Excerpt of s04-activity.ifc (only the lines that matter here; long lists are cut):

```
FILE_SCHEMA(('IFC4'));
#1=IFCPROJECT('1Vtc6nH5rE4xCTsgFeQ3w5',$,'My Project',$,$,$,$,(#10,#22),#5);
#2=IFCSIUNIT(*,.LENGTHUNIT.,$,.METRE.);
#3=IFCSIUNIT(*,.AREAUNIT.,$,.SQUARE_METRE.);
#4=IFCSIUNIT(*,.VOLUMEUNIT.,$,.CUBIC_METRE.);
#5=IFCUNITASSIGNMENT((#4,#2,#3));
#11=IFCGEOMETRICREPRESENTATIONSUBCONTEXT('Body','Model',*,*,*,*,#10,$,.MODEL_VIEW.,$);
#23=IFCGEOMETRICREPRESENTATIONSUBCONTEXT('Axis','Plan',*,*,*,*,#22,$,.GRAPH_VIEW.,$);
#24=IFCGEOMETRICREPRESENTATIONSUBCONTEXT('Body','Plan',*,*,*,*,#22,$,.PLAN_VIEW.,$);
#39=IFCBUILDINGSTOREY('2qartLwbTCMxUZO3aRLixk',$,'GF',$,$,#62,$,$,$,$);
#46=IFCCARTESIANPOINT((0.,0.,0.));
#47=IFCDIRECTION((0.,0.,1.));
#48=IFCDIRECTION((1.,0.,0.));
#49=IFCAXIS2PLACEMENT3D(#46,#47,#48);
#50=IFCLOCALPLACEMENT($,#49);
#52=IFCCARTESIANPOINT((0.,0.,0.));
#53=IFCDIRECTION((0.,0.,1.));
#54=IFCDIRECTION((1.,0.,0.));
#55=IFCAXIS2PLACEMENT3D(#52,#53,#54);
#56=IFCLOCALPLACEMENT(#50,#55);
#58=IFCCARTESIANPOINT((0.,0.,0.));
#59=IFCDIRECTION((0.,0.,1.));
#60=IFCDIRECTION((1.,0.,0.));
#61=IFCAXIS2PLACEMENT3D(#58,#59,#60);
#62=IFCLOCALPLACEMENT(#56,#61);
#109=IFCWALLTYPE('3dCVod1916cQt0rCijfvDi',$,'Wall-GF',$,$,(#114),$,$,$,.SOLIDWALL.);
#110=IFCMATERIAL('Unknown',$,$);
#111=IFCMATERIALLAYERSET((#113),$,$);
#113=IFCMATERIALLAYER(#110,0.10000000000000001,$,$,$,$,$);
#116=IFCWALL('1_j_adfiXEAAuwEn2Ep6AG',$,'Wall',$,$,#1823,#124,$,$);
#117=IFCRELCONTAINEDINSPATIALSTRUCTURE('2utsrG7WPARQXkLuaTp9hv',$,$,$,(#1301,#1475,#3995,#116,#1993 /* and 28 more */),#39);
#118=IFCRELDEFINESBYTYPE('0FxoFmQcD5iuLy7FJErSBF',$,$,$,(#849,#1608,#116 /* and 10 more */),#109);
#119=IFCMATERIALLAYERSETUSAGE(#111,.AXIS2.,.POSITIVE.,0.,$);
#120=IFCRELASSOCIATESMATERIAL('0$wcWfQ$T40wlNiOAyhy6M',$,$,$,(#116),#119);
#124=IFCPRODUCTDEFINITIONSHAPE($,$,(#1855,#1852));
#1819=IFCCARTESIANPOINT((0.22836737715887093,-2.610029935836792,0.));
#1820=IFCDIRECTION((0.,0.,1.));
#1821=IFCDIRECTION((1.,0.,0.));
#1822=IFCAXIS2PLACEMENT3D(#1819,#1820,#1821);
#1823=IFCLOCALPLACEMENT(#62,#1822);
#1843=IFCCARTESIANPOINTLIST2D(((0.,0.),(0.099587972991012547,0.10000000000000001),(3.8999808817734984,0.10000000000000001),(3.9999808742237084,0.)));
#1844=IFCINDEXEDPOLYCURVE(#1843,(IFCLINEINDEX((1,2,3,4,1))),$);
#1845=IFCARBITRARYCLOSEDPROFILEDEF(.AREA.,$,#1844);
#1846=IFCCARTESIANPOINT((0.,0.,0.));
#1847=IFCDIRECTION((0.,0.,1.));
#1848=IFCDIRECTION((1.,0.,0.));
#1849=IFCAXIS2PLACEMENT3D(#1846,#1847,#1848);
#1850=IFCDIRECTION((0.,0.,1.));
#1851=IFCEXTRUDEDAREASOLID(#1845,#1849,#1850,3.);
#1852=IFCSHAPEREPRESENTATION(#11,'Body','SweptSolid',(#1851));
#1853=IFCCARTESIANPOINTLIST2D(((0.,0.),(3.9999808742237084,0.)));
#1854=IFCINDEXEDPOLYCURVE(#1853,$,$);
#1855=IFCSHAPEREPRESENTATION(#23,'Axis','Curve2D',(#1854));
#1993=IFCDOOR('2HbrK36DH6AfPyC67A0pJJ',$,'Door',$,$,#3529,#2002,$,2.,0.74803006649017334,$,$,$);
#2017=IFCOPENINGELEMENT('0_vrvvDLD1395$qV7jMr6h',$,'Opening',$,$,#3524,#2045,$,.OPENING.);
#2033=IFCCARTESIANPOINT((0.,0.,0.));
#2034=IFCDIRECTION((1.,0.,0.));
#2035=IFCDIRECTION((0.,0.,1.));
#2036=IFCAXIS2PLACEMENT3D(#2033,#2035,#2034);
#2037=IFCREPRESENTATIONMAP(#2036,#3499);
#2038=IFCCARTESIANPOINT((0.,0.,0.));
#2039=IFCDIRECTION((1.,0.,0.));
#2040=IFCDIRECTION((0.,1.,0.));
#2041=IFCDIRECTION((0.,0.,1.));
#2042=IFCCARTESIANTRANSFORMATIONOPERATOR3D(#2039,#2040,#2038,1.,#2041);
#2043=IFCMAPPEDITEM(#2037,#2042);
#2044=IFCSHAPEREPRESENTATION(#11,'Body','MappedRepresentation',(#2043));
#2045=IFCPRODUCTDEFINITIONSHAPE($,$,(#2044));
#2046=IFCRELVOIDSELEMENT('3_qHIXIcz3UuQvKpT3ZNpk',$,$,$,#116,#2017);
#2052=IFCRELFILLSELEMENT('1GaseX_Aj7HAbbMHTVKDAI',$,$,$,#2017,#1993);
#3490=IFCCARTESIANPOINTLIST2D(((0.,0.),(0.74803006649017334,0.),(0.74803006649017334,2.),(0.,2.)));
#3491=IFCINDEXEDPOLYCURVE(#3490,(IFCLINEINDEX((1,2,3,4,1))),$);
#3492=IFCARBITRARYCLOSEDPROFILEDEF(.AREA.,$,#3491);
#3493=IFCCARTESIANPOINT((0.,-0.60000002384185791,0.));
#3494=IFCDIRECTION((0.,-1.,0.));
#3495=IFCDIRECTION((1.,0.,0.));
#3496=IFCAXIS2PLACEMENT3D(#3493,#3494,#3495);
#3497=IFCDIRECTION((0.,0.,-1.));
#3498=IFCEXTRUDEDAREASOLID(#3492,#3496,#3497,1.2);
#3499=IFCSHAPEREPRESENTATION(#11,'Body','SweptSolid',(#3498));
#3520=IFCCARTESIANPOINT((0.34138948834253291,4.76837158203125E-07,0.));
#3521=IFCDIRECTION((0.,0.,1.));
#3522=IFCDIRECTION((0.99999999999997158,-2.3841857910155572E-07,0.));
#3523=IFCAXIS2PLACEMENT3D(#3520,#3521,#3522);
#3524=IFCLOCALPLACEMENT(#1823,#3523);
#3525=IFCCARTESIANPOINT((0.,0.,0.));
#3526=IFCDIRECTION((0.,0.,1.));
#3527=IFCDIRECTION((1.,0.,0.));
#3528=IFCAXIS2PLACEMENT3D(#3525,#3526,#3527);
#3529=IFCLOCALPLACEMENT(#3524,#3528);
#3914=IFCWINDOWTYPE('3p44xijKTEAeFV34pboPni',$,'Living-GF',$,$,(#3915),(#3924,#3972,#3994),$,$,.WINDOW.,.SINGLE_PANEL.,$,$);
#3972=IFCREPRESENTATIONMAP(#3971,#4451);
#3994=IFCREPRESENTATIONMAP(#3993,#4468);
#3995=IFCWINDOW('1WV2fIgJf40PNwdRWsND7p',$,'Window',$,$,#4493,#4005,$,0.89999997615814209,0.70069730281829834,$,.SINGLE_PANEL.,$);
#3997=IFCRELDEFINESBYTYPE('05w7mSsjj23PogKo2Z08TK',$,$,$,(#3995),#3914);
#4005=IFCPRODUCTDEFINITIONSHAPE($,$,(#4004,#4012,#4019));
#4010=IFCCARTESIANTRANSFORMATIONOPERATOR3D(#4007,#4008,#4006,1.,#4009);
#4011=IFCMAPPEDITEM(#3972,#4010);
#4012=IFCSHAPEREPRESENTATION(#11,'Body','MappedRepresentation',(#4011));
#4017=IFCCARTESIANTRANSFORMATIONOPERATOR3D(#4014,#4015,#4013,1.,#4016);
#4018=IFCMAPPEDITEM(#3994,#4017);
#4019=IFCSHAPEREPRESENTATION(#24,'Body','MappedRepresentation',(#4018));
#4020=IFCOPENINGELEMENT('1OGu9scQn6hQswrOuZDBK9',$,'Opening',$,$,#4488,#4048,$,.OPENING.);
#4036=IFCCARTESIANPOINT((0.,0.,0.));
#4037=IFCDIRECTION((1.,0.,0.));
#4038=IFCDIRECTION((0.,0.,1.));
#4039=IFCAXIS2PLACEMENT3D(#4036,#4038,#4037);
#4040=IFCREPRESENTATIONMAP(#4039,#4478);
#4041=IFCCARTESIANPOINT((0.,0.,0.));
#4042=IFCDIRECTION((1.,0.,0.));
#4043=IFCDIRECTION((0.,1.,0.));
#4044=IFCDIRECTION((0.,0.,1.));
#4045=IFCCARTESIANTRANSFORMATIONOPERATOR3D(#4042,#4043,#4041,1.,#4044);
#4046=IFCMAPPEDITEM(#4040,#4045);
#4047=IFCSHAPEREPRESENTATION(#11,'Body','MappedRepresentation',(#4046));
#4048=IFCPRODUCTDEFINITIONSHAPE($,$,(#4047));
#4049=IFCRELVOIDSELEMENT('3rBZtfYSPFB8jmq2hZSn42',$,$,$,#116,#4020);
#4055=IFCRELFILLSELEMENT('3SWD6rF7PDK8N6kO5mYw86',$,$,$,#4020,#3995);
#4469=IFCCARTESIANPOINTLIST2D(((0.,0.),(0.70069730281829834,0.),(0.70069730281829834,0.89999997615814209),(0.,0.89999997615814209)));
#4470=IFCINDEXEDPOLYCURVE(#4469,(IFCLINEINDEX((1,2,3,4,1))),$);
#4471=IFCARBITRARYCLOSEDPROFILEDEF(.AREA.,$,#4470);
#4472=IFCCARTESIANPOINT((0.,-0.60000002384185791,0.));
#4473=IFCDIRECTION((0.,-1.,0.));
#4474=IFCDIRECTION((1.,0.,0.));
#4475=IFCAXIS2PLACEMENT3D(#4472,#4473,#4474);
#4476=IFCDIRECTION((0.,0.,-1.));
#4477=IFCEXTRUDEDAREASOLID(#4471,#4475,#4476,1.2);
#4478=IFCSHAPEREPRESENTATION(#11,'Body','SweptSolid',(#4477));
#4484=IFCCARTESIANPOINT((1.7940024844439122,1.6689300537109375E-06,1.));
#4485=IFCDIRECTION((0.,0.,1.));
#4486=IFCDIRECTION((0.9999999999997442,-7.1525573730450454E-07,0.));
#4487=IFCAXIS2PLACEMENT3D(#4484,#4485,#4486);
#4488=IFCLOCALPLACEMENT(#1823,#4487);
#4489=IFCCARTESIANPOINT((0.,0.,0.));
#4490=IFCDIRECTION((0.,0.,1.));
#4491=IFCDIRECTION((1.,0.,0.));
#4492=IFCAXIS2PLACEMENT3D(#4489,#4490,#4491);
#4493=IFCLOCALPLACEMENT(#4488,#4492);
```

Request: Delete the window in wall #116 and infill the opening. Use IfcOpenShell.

```python
import ifcopenshell
import ifcopenshell.api.feature
import ifcopenshell.api.root
import ifcopenshell.geom
import ifcopenshell.util.shape

model = ifcopenshell.open("s04-activity.ifc")
settings = ifcopenshell.geom.settings()


def volume(element):
    """Net volume in cubic metres, openings subtracted."""
    shape = ifcopenshell.geom.create_shape(settings, element)
    return ifcopenshell.util.shape.get_volume(shape.geometry)


window = model.by_guid("1WV2fIgJf40PNwdRWsND7p")
opening = window.FillsVoids[0].RelatingOpeningElement
wall = opening.VoidsElements[0].RelatingBuildingElement
before = volume(wall)

ifcopenshell.api.root.remove_product(model, product=window)
ifcopenshell.api.feature.remove_feature(model, feature=opening)

after = volume(wall)

print(f"wall volume {before:.3f} -> {after:.3f} m3")

model.write("s04-activity_edited.ifc")
```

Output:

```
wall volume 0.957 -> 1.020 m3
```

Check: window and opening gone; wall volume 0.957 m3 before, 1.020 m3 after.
